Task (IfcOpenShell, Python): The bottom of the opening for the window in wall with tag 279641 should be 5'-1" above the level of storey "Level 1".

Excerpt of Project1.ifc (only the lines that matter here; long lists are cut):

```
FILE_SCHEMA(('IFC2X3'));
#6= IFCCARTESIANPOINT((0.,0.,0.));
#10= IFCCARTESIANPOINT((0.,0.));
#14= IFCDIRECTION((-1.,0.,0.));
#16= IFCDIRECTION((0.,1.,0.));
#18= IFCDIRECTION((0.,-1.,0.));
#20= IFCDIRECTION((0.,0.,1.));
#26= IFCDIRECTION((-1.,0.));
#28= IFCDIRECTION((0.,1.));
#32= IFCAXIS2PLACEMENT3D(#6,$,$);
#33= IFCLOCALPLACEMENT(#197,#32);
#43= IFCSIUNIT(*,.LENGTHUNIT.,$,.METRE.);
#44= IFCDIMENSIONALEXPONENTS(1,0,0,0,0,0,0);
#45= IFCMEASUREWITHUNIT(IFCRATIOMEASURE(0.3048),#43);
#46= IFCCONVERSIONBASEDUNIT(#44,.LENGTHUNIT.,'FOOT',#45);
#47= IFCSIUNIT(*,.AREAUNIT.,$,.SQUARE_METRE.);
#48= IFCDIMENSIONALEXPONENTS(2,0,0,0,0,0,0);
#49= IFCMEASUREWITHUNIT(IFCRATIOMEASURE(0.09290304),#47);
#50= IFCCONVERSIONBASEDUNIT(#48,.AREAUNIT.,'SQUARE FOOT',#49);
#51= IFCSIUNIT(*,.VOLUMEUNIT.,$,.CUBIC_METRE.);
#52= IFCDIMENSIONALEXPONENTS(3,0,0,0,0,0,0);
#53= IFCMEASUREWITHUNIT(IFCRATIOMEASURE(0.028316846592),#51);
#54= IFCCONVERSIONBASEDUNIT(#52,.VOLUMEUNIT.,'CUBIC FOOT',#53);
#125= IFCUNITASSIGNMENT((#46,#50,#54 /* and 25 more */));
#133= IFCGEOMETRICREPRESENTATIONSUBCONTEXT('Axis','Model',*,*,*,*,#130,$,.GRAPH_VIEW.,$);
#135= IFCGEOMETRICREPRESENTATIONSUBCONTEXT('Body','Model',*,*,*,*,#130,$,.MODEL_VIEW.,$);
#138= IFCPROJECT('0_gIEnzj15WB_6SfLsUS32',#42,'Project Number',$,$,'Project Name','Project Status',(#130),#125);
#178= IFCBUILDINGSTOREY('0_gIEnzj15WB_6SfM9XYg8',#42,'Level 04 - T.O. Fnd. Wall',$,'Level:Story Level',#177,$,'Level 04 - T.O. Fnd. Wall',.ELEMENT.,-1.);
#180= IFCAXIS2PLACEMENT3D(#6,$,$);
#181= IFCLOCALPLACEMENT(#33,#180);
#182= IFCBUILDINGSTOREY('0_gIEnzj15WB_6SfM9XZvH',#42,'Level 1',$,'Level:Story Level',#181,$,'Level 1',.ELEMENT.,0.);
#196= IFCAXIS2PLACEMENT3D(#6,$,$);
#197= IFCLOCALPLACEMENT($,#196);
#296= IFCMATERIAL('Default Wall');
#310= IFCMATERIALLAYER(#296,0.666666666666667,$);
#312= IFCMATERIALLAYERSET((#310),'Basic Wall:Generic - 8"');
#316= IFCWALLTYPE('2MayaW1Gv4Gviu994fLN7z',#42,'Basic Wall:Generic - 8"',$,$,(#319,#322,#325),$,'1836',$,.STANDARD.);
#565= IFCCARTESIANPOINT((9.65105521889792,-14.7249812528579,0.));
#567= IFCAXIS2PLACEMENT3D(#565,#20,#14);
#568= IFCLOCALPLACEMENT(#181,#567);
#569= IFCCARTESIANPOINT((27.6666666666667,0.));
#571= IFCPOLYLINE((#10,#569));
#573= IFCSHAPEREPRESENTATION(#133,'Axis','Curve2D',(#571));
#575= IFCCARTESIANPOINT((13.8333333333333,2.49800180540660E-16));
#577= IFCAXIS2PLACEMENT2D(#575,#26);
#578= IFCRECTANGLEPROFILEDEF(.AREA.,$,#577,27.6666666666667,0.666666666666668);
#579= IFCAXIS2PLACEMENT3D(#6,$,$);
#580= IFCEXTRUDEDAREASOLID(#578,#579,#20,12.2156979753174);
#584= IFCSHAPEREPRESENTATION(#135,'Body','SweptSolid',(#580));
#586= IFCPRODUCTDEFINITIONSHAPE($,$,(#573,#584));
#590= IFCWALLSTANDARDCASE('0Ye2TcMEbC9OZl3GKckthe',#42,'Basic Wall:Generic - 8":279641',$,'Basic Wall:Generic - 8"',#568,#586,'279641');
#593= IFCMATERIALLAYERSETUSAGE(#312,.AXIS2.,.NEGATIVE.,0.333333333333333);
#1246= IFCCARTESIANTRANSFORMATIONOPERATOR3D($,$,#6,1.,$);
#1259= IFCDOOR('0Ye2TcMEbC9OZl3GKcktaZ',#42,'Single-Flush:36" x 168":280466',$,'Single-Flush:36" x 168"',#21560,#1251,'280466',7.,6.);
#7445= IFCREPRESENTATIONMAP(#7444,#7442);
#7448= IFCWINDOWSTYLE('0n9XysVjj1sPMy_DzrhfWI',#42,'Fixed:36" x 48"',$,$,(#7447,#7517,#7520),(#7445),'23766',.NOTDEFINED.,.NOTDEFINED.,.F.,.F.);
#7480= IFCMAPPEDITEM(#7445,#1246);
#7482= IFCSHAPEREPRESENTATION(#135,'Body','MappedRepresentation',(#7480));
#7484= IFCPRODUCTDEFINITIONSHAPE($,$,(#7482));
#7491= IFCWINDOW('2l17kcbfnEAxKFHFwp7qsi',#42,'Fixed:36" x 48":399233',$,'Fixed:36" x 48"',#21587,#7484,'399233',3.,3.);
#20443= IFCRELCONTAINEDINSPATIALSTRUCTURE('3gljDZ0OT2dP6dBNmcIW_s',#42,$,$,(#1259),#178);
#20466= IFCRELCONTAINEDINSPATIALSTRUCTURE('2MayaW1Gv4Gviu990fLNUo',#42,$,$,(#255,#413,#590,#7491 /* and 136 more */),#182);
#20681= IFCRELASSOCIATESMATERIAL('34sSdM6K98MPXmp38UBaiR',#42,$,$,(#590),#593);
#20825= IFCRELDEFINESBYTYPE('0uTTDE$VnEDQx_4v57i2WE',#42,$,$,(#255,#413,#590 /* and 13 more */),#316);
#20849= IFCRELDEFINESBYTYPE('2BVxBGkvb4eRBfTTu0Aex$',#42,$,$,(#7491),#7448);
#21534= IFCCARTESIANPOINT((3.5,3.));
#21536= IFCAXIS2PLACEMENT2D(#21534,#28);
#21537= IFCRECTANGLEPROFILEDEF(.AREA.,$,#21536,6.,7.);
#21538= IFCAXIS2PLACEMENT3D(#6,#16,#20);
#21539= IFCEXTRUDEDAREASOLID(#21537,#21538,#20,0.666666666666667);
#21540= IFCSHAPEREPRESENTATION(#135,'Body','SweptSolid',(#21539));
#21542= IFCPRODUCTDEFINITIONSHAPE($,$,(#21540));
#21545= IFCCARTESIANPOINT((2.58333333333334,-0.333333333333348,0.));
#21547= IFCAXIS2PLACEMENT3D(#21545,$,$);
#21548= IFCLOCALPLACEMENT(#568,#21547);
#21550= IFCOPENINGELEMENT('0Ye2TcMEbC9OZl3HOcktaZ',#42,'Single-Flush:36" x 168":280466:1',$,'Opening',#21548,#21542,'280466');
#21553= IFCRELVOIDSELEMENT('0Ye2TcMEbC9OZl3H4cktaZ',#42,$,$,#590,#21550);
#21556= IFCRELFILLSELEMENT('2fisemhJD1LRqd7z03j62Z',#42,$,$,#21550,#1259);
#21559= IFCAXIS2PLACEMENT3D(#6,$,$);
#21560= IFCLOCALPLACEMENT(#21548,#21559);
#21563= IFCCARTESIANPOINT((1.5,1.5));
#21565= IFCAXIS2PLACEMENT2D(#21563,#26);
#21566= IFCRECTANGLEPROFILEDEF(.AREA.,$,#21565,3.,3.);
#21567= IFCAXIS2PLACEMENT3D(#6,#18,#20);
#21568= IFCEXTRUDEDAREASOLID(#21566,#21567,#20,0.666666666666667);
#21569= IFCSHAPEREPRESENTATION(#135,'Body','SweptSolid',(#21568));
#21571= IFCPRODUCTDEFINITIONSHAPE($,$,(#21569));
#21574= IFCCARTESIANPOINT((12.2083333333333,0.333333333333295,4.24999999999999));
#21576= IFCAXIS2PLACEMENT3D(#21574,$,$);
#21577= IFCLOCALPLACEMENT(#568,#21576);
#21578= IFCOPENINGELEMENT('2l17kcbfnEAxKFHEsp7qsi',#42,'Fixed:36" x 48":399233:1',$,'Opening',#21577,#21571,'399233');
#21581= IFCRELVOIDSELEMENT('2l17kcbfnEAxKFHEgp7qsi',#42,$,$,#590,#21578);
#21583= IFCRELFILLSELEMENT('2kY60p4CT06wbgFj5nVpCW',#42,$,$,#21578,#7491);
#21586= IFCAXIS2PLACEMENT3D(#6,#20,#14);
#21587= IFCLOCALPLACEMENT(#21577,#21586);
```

```python
import numpy as np
import ifcopenshell
import ifcopenshell.api.geometry
import ifcopenshell.geom
import ifcopenshell.util.element
import ifcopenshell.util.placement
import ifcopenshell.util.shape
import ifcopenshell.util.unit

model = ifcopenshell.open("Project1.ifc")
unit_scale = ifcopenshell.util.unit.calculate_unit_scale(model)

window = model.by_id(7491)
opening = window.FillsVoids[0].RelatingOpeningElement
storey = ifcopenshell.util.element.get_container(window, ifc_class="IfcBuildingStorey")
level = ifcopenshell.util.placement.get_local_placement(storey.ObjectPlacement)[2, 3]

# The opening's origin need not be at the sill, so measure its lowest point.
shape = ifcopenshell.geom.create_shape(ifcopenshell.geom.settings(), opening)
bottom = ifcopenshell.util.shape.get_shape_bottom_elevation(shape, shape.geometry) / unit_scale
dz = level + 61 * 0.0254 / unit_scale - bottom

shift = np.array([0.0, 0.0, dz])
# The window is placed relative to its opening, so it follows when the opening moves.
matrix = ifcopenshell.util.placement.get_local_placement(opening.ObjectPlacement)
matrix[:3, 3] += shift
ifcopenshell.api.geometry.edit_object_placement(
    model, product=opening, matrix=matrix, is_si=False, should_transform_children=True
)

print(f"moved by {dz * unit_scale:+.3f} m")

model.write("Project1_rev.ifc")
```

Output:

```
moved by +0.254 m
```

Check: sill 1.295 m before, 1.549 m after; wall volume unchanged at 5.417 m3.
